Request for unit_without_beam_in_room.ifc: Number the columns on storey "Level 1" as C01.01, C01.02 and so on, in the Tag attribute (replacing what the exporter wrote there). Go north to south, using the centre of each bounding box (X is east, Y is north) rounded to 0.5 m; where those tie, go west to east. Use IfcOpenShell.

First a look at what the model holds.

```python
import ifcopenshell
import ifcopenshell.util.element
import ifcopenshell.util.placement

model = ifcopenshell.open("unit_without_beam_in_room.ifc")
print(model.schema)
storey = next(s for s in model.by_type("IfcBuildingStorey") if s.Name == "Level 1")
columns = [e for e in ifcopenshell.util.element.get_decomposition(storey) if e.is_a("IfcColumn")]
for e in sorted(columns, key=lambda e: e.id()):
    origin = ifcopenshell.util.placement.get_local_placement(e.ObjectPlacement)[:3, 3]
    print(e.id(), e.Tag, e.Name, origin.round(2) + 0.0, sep=" | ")
```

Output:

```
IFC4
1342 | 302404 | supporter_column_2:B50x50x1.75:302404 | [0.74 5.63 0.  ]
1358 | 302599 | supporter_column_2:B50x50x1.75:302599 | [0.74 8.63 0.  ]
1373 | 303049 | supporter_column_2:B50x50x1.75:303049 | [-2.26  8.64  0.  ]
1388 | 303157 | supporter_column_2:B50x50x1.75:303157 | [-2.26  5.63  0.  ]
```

```python
import ifcopenshell
import ifcopenshell.geom
import ifcopenshell.util.element
import ifcopenshell.util.shape

model = ifcopenshell.open("unit_without_beam_in_room.ifc")
settings = ifcopenshell.geom.settings()
settings.set("use-world-coords", True)


def centre(element):
    shape = ifcopenshell.geom.create_shape(settings, element)
    return ifcopenshell.util.shape.get_bbox_centroid(shape.geometry)


storey = next(s for s in model.by_type("IfcBuildingStorey") if s.Name == "Level 1")
columns = [e for e in ifcopenshell.util.element.get_decomposition(storey) if e.is_a("IfcColumn")]

# Insertion points can sit at a corner or the storey origin, so sort by the geometry (in metres).
centres = {e: centre(e) for e in columns}
columns.sort(key=lambda e: (-round(centres[e][1] / 0.5), centres[e][0]))

for i, e in enumerate(columns, start=1):
    number = f"C01.{i:02d}"
    e.Tag = number
    print(e.id(), number)

model.write("unit_without_beam_in_room_rev.ifc")
```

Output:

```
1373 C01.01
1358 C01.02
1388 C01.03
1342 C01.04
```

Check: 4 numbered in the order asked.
